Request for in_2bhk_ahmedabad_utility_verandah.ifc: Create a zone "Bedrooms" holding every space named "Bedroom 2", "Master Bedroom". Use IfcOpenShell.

First a look at what the model holds.

```python
import ifcopenshell

model = ifcopenshell.open("in_2bhk_ahmedabad_utility_verandah.ifc")
print(model.schema)
seen = {}
for space in model.by_type("IfcSpace"):
    seen[space.LongName] = seen.get(space.LongName, 0) + 1
for name, count in sorted(seen.items(), key=str):
    print(count, "x", name)
print("zones:", [z.Name for z in model.by_type("IfcZone")][:20])
```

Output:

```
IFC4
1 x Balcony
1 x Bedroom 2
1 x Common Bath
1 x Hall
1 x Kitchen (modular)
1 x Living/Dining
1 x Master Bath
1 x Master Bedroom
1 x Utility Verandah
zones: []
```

```python
import ifcopenshell
import ifcopenshell.api.group
import ifcopenshell.api.root

model = ifcopenshell.open("in_2bhk_ahmedabad_utility_verandah.ifc")

names = {"Bedroom 2", "Master Bedroom"}
spaces = [s for s in model.by_type("IfcSpace") if s.LongName in names]

zone = ifcopenshell.api.root.create_entity(model, ifc_class="IfcZone", name="Bedrooms")
ifcopenshell.api.group.assign_group(model, products=spaces, group=zone)
print(len(spaces), "spaces in", zone.Name)

model.write("in_2bhk_ahmedabad_utility_verandah-out.ifc")
```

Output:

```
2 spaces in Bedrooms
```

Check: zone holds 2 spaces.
